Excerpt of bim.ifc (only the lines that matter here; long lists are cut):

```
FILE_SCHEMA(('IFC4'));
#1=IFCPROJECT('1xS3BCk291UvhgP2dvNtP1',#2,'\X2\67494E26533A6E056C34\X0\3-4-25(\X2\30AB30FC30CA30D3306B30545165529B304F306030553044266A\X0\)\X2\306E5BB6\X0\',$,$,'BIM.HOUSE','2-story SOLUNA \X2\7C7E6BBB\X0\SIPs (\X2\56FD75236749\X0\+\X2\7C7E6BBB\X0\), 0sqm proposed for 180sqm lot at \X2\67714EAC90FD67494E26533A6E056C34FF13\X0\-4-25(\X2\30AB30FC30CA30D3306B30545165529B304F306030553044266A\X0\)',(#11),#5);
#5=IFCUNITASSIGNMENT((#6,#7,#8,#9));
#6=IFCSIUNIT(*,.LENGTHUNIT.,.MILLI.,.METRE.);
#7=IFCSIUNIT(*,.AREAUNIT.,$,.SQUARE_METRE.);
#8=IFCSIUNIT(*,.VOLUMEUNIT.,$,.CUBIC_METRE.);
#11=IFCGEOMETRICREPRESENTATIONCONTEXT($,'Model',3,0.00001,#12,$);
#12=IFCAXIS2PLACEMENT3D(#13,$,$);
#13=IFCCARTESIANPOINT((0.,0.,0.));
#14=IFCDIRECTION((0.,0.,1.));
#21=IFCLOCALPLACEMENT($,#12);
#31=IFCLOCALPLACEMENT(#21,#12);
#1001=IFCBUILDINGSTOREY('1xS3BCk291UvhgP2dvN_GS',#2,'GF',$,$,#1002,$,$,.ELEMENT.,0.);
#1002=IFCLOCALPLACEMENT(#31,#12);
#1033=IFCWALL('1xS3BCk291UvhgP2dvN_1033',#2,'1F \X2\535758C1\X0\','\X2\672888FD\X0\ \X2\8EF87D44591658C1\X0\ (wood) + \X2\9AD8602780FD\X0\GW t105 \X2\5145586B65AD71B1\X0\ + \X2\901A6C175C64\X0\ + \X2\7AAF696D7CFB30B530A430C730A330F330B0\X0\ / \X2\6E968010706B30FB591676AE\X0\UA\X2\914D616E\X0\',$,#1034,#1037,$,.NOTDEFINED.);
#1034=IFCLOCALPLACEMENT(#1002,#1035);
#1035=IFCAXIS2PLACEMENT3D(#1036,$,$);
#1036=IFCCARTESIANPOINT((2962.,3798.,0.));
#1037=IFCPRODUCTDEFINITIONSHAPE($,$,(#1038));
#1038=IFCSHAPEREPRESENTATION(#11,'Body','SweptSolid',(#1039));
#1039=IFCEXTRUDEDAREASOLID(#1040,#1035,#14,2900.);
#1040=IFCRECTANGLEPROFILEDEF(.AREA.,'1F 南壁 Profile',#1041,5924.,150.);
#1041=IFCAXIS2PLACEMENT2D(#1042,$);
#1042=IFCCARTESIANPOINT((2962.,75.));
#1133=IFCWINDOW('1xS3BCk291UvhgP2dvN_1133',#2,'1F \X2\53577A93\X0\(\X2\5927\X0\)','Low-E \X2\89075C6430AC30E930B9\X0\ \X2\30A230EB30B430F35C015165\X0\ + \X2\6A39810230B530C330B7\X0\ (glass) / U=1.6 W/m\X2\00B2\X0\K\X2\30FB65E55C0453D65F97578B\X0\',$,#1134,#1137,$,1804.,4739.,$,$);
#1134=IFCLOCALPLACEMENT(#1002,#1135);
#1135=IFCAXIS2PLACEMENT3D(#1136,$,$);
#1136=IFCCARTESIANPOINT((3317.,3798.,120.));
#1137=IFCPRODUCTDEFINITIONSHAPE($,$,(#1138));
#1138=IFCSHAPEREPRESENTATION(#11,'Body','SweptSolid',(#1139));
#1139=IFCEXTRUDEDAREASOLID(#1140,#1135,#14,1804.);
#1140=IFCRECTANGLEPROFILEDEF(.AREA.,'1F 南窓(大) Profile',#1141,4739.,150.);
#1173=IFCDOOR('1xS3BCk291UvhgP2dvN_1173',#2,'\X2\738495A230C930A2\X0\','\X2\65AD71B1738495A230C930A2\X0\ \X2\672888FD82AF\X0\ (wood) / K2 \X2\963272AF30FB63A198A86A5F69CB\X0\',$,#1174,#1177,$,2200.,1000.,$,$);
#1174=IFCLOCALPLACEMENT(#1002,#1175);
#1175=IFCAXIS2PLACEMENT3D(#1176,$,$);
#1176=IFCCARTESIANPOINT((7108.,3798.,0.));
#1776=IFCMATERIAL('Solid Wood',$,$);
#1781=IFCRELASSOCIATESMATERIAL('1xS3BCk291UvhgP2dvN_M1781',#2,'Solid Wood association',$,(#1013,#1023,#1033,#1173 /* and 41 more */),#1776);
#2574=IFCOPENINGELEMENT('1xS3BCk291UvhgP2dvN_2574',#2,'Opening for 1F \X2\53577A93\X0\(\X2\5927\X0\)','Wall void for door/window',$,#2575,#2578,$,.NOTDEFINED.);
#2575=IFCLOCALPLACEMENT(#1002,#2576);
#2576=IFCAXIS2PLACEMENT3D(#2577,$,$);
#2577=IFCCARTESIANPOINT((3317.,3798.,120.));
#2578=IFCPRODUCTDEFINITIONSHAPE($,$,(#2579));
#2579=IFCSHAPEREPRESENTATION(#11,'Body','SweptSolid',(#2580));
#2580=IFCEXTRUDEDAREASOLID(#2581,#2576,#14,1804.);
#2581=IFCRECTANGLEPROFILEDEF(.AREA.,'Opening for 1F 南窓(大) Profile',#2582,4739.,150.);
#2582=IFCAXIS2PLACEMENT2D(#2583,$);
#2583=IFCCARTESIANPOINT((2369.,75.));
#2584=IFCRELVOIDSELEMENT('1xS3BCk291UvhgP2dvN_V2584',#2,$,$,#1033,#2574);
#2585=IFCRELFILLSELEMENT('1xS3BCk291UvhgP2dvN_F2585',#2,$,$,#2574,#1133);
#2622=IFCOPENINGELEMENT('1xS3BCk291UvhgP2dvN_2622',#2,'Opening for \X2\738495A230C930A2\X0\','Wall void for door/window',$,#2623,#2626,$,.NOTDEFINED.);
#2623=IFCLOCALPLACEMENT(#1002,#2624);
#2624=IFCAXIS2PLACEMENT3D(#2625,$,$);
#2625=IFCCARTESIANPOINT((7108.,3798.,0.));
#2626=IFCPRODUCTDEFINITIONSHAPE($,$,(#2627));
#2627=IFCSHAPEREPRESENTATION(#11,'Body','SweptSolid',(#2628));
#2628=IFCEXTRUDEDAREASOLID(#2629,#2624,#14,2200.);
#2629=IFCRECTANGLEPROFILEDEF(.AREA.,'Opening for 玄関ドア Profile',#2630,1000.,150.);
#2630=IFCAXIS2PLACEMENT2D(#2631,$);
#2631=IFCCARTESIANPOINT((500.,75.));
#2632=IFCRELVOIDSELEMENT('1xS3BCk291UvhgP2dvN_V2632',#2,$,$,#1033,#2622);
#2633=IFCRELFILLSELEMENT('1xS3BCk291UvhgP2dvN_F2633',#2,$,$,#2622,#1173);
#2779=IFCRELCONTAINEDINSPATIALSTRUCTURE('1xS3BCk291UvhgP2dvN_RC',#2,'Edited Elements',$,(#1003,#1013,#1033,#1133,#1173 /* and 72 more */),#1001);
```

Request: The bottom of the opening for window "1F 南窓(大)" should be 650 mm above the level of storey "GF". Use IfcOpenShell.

```python
import numpy as np
import ifcopenshell
import ifcopenshell.api.geometry
import ifcopenshell.geom
import ifcopenshell.util.element
import ifcopenshell.util.placement
import ifcopenshell.util.shape
import ifcopenshell.util.unit

model = ifcopenshell.open("bim.ifc")
unit_scale = ifcopenshell.util.unit.calculate_unit_scale(model)

window = model.by_id(1133)
opening = window.FillsVoids[0].RelatingOpeningElement
storey = ifcopenshell.util.element.get_container(window, ifc_class="IfcBuildingStorey")
level = ifcopenshell.util.placement.get_local_placement(storey.ObjectPlacement)[2, 3]

# The opening's origin need not be at the sill, so measure its lowest point.
shape = ifcopenshell.geom.create_shape(ifcopenshell.geom.settings(), opening)
bottom = ifcopenshell.util.shape.get_shape_bottom_elevation(shape, shape.geometry) / unit_scale
dz = level + 650.0 - bottom

shift = np.array([0.0, 0.0, dz])
# The window is not placed relative to its opening, so move both.
for product in (opening, window):
    matrix = ifcopenshell.util.placement.get_local_placement(product.ObjectPlacement)
    matrix[:3, 3] += shift
    ifcopenshell.api.geometry.edit_object_placement(model, product=product, matrix=matrix, is_si=False)

print(f"moved by {dz * unit_scale:+.3f} m")

model.write("bim_edited.ifc")
```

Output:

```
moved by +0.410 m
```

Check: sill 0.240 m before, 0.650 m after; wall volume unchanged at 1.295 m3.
